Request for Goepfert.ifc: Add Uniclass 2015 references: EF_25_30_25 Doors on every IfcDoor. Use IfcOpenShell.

First a look at what the model holds.

```python
import ifcopenshell

model = ifcopenshell.open("Goepfert.ifc")
print(model.schema)
print("classifications:", [c.Name for c in model.by_type("IfcClassification")])
for ifc_class in ("IfcDoor", "IfcRoof", "IfcStair", "IfcWall", "IfcWindow"):
    print(ifc_class, len(model.by_type(ifc_class)))
```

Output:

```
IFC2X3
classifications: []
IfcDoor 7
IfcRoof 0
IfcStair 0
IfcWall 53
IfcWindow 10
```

```python
import ifcopenshell
import ifcopenshell.api.classification

model = ifcopenshell.open("Goepfert.ifc")

# IFC2X3 requires Source and Edition and has no link from the project to the system.
system = model.create_entity("IfcClassification", Source="NBS", Edition="2015", Name="Uniclass 2015")

codes = {
    "IfcDoor": ("EF_25_30_25", "Doors"),
}
for ifc_class, (code, name) in codes.items():
    products = model.by_type(ifc_class)
    ifcopenshell.api.classification.add_reference(
        model, products=products, classification=system, identification=code, name=name
    )
    print(code, len(products))

model.write("Goepfert_rev.ifc")
```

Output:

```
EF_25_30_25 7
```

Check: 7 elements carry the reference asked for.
